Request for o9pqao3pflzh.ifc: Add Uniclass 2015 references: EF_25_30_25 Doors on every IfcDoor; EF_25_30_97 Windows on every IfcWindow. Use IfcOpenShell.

First a look at what the model holds.

```python
import ifcopenshell

model = ifcopenshell.open("o9pqao3pflzh.ifc")
print(model.schema)
print("classifications:", [c.Name for c in model.by_type("IfcClassification")])
for ifc_class in ("IfcDoor", "IfcRoof", "IfcStair", "IfcWall", "IfcWindow"):
    print(ifc_class, len(model.by_type(ifc_class)))
```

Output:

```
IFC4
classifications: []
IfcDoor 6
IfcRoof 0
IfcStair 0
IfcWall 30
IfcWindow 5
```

```python
import ifcopenshell
import ifcopenshell.api.classification

model = ifcopenshell.open("o9pqao3pflzh.ifc")

system = ifcopenshell.api.classification.add_classification(model, classification="Uniclass 2015")

codes = {
    "IfcDoor": ("EF_25_30_25", "Doors"),
    "IfcWindow": ("EF_25_30_97", "Windows"),
}
for ifc_class, (code, name) in codes.items():
    products = model.by_type(ifc_class)
    ifcopenshell.api.classification.add_reference(
        model, products=products, classification=system, identification=code, name=name
    )
    print(code, len(products))

model.write("o9pqao3pflzh_v2.ifc")
```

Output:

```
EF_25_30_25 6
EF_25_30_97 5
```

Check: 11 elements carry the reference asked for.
